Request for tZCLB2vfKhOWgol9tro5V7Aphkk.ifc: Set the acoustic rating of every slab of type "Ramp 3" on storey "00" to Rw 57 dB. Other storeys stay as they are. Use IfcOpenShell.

First a look at what the model holds.

```python
import ifcopenshell
import ifcopenshell.util.element

model = ifcopenshell.open("tZCLB2vfKhOWgol9tro5V7Aphkk.ifc")
print(model.schema)
storey = next(s for s in model.by_type("IfcBuildingStorey") if s.Name == "00")
slabs = [e for e in ifcopenshell.util.element.get_decomposition(storey) if e.is_a("IfcSlab")]
seen = {}
for e in slabs:
    element_type = ifcopenshell.util.element.get_type(e)
    key = (element_type.Name if element_type != e and element_type else None, ifcopenshell.util.element.get_pset(e, "Pset_SlabCommon", "AcousticRating"))
    seen[key] = seen.get(key, 0) + 1
for (name, value), count in sorted(seen.items(), key=str):
    print(count, "x", name, "|", value)
```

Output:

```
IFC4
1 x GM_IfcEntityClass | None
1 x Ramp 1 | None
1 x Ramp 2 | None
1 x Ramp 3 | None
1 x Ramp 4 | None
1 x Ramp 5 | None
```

```python
import ifcopenshell
import ifcopenshell.api.pset
import ifcopenshell.util.element

model = ifcopenshell.open("tZCLB2vfKhOWgol9tro5V7Aphkk.ifc")

storey = next(s for s in model.by_type("IfcBuildingStorey") if s.Name == "00")
slabs = [e for e in ifcopenshell.util.element.get_decomposition(storey) if e.is_a("IfcSlab")]

count = 0
for e in slabs:
    element_type = ifcopenshell.util.element.get_type(e)
    if element_type in (None, e) or element_type.Name != "Ramp 3":
        continue
    # add_pset returns the element's existing set when there is one.
    pset = ifcopenshell.api.pset.add_pset(model, product=e, name="Pset_SlabCommon")
    ifcopenshell.api.pset.edit_pset(model, pset=pset, properties={"AcousticRating": "Rw 57 dB"})
    count += 1

print(count, "slabs updated")

model.write("tZCLB2vfKhOWgol9tro5V7Aphkk_updated.ifc")
```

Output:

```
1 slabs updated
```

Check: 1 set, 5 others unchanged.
